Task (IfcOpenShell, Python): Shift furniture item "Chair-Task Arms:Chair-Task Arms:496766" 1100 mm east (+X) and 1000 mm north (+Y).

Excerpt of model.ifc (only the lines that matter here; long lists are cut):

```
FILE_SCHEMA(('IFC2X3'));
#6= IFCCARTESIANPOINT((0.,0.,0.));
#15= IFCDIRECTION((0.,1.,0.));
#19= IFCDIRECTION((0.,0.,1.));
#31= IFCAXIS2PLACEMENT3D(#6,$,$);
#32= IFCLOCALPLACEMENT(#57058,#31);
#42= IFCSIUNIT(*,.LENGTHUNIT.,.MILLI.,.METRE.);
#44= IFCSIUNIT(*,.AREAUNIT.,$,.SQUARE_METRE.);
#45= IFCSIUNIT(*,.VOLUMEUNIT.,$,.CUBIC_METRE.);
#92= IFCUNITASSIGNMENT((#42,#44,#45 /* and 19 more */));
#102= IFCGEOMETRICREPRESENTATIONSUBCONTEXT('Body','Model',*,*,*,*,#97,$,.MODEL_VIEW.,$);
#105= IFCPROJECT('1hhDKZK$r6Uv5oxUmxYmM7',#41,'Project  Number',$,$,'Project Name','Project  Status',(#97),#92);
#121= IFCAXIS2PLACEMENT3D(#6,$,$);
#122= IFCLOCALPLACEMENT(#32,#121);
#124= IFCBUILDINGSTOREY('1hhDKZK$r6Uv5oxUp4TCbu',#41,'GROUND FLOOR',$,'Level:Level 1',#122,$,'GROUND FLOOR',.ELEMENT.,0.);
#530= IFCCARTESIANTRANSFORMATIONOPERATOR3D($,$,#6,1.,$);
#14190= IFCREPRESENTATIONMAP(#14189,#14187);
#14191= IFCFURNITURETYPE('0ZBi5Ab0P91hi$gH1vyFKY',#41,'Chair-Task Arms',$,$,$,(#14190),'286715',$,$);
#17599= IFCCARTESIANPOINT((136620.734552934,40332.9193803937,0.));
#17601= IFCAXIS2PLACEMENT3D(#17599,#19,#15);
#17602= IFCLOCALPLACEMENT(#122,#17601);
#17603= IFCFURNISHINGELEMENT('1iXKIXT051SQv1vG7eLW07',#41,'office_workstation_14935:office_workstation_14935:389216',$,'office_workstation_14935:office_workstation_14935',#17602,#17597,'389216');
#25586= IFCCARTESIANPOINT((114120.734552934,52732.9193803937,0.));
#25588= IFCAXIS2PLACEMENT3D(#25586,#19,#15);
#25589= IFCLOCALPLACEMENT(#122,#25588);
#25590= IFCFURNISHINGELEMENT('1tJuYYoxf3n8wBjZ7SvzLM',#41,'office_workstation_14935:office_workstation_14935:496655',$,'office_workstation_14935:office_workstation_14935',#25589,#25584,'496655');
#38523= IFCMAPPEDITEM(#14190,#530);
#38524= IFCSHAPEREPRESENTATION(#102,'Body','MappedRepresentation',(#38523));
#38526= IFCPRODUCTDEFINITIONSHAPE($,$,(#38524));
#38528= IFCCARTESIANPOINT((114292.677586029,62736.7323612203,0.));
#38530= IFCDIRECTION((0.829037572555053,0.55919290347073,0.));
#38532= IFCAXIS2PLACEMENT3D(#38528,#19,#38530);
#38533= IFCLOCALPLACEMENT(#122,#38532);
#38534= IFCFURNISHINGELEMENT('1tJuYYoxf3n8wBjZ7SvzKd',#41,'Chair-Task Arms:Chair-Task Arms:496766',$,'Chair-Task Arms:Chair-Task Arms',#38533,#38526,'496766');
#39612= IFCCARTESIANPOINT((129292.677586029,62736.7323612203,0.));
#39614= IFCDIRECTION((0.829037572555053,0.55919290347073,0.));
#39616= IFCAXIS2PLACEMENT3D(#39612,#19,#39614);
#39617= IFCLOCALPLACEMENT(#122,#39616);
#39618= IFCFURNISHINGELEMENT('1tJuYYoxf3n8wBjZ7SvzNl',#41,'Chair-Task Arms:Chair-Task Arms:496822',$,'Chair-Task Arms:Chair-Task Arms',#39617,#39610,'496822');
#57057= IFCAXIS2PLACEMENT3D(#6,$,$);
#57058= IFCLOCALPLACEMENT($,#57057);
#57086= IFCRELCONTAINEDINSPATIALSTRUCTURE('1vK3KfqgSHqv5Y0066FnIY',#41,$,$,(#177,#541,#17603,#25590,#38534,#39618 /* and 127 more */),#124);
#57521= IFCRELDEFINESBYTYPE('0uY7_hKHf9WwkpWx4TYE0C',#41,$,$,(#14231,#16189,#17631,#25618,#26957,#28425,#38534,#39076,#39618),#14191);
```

```python
import ifcopenshell
import ifcopenshell.api.geometry
import ifcopenshell.util.placement

model = ifcopenshell.open("model.ifc")

item = model.by_id(38534)
matrix = ifcopenshell.util.placement.get_local_placement(item.ObjectPlacement)
matrix[0, 3] += 1100.0
matrix[1, 3] += 1000.0
ifcopenshell.api.geometry.edit_object_placement(model, product=item, matrix=matrix, is_si=False)

print(ifcopenshell.util.placement.get_local_placement(item.ObjectPlacement).round(3) + 0.0)

model.write("model_rev.ifc")
```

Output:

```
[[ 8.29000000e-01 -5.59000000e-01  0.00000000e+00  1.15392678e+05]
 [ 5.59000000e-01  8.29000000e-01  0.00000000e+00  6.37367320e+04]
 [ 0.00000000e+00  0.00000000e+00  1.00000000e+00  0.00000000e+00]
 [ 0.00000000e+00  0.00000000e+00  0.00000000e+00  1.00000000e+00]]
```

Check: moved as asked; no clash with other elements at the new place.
